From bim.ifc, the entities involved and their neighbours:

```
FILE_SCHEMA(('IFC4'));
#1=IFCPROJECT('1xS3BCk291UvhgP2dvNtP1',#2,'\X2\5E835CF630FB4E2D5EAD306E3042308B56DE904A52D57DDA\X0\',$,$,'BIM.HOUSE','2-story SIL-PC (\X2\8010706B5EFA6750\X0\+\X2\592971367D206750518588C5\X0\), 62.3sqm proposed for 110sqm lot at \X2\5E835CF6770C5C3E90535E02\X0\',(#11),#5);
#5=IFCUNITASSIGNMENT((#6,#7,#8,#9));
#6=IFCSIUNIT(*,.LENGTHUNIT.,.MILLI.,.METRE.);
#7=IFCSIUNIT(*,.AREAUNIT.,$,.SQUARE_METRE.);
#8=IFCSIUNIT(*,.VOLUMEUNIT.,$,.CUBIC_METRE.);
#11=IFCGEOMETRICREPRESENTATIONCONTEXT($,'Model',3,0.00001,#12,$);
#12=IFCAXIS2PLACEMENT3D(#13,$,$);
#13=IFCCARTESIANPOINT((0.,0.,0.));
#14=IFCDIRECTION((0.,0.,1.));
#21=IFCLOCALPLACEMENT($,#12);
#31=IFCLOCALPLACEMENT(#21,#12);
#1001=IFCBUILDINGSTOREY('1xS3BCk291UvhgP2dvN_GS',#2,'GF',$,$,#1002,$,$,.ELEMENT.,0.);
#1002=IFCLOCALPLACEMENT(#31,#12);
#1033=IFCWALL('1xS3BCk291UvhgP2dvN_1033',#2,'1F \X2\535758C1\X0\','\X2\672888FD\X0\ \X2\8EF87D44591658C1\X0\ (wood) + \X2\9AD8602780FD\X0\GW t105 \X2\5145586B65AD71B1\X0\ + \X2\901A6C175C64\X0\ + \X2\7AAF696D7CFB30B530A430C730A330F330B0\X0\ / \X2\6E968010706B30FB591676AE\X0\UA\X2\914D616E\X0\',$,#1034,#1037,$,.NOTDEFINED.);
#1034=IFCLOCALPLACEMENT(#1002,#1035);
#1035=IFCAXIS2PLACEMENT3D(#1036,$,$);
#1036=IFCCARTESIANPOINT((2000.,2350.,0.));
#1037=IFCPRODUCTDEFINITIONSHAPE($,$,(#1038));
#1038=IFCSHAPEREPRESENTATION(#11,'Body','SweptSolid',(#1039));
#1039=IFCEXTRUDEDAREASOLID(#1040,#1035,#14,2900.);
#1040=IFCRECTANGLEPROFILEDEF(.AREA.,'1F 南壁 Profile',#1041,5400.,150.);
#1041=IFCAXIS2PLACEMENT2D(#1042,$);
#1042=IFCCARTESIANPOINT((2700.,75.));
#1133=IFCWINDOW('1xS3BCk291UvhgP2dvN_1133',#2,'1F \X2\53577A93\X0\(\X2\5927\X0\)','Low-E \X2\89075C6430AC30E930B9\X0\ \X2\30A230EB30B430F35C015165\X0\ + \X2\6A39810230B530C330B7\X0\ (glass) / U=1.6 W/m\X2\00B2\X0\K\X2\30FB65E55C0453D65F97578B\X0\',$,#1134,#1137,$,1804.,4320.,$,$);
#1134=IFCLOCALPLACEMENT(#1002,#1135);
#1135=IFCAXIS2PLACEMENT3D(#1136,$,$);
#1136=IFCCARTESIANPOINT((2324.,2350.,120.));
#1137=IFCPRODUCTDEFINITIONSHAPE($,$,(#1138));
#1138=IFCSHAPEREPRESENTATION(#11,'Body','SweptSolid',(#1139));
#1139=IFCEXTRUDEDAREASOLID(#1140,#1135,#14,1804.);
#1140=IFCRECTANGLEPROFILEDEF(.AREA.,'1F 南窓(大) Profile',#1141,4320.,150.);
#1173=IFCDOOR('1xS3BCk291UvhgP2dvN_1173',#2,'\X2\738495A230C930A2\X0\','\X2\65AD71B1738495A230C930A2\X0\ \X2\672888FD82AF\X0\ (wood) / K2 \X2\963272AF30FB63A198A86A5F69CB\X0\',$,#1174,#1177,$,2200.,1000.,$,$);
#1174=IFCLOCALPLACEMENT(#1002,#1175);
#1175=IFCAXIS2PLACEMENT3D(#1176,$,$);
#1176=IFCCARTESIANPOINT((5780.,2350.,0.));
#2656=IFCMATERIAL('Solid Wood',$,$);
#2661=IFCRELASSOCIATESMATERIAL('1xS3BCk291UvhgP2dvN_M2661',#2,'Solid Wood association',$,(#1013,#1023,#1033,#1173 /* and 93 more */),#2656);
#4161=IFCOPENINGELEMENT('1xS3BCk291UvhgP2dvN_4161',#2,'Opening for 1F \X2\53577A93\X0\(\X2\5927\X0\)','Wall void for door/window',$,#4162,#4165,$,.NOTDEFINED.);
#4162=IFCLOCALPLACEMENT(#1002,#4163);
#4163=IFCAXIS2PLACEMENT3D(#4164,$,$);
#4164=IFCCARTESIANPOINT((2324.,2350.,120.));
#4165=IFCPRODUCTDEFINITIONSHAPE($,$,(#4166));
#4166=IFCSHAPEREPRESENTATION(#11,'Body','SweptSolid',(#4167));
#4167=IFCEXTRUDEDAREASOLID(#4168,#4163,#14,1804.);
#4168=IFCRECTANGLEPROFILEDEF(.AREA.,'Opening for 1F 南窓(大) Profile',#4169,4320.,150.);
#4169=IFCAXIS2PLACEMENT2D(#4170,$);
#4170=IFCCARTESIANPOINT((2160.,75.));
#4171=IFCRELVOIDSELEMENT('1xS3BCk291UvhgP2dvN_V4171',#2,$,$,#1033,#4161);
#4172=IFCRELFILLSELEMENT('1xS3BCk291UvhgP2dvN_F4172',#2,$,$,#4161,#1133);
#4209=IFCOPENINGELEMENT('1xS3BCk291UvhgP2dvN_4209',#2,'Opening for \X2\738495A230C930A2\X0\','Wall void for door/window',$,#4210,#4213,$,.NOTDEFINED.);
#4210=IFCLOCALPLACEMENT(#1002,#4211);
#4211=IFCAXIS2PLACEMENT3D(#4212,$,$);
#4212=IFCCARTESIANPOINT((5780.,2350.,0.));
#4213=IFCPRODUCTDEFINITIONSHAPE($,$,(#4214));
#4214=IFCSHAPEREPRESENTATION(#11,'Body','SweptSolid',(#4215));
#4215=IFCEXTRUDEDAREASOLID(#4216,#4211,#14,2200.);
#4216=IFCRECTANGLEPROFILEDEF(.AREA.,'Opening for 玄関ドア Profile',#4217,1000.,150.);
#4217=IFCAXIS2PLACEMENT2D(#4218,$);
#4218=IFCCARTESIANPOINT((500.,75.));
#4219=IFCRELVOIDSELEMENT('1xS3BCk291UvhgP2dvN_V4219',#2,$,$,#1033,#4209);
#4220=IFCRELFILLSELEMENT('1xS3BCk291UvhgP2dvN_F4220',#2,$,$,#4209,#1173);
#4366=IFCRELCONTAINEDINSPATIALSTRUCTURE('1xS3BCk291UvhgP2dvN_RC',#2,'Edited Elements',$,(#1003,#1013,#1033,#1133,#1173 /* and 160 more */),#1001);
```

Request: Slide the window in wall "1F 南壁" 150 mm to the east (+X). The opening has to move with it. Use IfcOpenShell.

```python
import ifcopenshell
import ifcopenshell.api.geometry
import ifcopenshell.util.placement
import ifcopenshell.util.unit

model = ifcopenshell.open("bim.ifc")
unit_scale = ifcopenshell.util.unit.calculate_unit_scale(model)

window = model.by_guid("1xS3BCk291UvhgP2dvN_1133")
opening = window.FillsVoids[0].RelatingOpeningElement
wall = opening.VoidsElements[0].RelatingBuildingElement

wall_matrix = ifcopenshell.util.placement.get_local_placement(wall.ObjectPlacement)
shift = wall_matrix[:3, 0] * 0.15 / unit_scale
before = ifcopenshell.util.placement.get_local_placement(window.ObjectPlacement)[:3, 3].copy()

# The window is not placed relative to its opening, so move both.
for product in (opening, window):
    matrix = ifcopenshell.util.placement.get_local_placement(product.ObjectPlacement)
    matrix[:3, 3] += shift
    ifcopenshell.api.geometry.edit_object_placement(model, product=product, matrix=matrix, is_si=False)

after = ifcopenshell.util.placement.get_local_placement(window.ObjectPlacement)[:3, 3]
print("window moved by", (after - before).round(3) + 0.0)

model.write("bim_rev.ifc")
```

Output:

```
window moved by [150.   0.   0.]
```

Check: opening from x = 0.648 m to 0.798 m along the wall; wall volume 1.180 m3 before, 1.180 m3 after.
